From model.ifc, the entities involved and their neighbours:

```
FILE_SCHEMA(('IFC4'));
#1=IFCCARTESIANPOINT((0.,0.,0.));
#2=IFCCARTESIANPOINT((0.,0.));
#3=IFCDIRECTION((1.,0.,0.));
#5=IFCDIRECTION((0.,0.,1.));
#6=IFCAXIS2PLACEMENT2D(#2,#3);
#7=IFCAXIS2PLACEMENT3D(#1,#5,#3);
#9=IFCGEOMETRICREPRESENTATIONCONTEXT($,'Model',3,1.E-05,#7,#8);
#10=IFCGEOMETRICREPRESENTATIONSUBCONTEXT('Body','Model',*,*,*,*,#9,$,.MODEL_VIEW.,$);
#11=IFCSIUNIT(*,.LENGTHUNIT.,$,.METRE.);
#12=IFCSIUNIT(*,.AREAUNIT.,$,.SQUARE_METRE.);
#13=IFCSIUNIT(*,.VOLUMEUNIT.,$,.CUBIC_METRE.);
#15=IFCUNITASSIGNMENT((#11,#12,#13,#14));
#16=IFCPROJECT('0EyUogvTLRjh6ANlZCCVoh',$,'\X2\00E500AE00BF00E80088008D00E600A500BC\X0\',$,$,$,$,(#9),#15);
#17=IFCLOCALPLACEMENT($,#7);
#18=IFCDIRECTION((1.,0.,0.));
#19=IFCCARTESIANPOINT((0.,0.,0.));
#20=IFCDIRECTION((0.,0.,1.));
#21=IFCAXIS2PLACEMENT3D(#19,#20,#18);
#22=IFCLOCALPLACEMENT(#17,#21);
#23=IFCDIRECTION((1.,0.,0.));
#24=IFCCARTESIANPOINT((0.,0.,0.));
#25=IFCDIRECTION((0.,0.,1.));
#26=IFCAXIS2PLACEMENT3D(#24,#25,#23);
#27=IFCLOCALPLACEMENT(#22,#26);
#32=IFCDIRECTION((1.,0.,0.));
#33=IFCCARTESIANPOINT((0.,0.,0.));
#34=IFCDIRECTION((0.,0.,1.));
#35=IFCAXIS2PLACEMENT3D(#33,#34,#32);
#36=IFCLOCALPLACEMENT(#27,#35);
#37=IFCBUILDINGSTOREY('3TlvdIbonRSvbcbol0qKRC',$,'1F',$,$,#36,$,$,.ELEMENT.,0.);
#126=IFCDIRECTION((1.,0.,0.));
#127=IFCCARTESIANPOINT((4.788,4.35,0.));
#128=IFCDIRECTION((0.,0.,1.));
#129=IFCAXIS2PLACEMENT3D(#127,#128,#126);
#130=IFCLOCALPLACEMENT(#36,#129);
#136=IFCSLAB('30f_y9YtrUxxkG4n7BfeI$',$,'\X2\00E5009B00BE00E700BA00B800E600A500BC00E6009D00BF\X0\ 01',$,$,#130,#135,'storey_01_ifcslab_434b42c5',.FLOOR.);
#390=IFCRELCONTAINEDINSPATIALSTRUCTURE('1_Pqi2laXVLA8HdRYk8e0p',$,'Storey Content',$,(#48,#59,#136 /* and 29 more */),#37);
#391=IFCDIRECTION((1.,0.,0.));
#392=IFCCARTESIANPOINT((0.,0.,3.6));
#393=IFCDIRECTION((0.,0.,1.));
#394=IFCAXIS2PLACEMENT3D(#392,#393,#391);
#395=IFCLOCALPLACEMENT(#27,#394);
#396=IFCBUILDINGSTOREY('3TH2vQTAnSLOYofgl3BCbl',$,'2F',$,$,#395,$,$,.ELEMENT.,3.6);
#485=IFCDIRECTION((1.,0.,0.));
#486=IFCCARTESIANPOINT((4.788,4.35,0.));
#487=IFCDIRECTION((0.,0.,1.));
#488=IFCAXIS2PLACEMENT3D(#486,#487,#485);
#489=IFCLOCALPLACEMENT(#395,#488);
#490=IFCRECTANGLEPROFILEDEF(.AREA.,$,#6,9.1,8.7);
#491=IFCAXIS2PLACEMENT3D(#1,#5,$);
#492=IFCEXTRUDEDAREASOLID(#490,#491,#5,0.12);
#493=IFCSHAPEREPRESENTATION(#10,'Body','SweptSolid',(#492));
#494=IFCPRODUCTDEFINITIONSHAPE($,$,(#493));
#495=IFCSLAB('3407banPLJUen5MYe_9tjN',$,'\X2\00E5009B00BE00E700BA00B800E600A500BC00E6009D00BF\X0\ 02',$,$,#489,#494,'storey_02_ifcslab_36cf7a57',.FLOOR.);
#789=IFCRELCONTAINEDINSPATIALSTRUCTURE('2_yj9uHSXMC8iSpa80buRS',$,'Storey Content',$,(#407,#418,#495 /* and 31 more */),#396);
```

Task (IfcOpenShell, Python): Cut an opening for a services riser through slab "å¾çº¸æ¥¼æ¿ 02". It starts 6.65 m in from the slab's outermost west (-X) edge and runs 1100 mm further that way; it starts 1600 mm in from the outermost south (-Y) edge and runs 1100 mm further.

```python
import numpy as np
import ifcopenshell
import ifcopenshell.api.feature
import ifcopenshell.api.geometry
import ifcopenshell.api.root
import ifcopenshell.geom
import ifcopenshell.util.placement
import ifcopenshell.util.representation
import ifcopenshell.util.shape
import ifcopenshell.util.unit

model = ifcopenshell.open("model.ifc")
unit_scale = ifcopenshell.util.unit.calculate_unit_scale(model)
settings = ifcopenshell.geom.settings()


def volume(element):
    """Net volume in cubic metres, openings subtracted."""
    shape = ifcopenshell.geom.create_shape(settings, element)
    return ifcopenshell.util.shape.get_volume(shape.geometry)


slab = model.by_id(495)
before = volume(slab)

# Extent in the slab's own axes, in metres. The edges named are its -X and -Y sides.
slab_shape = ifcopenshell.geom.create_shape(settings, slab)
vertices = ifcopenshell.util.shape.get_vertices(slab_shape.geometry)
x_min, y_min, bottom = vertices.min(axis=0)
top = vertices[:, 2].max()

opening = ifcopenshell.api.root.create_entity(model, ifc_class="IfcOpeningElement", name="Services riser opening", predefined_type="OPENING")
context = ifcopenshell.util.representation.get_context(model, "Model", "Body", "MODEL_VIEW")
width, depth = 1.1, 1.1
outline = [(0.0, 0.0), (width, 0.0), (width, depth), (0.0, depth), (0.0, 0.0)]
# Overshoot both faces by 50 mm so the cut is clean.
shape = ifcopenshell.api.geometry.add_slab_representation(
    model, context=context, depth=top - bottom + 0.1, polyline=outline
)
ifcopenshell.api.geometry.assign_representation(model, product=opening, representation=shape)

matrix = ifcopenshell.util.placement.get_local_placement(slab.ObjectPlacement)
matrix[:, 3] = matrix @ np.append(np.array([x_min + 6.65, y_min + 1.6, bottom - 0.05]) / unit_scale, 1.0)
ifcopenshell.api.geometry.edit_object_placement(model, product=opening, matrix=matrix, is_si=False)
ifcopenshell.api.feature.add_feature(model, feature=opening, element=slab)

after = volume(slab)

print(f"slab volume {before:.3f} -> {after:.3f} m3")

model.write("model_updated.ifc")
```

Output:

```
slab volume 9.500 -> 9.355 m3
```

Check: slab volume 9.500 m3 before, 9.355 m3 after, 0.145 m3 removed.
